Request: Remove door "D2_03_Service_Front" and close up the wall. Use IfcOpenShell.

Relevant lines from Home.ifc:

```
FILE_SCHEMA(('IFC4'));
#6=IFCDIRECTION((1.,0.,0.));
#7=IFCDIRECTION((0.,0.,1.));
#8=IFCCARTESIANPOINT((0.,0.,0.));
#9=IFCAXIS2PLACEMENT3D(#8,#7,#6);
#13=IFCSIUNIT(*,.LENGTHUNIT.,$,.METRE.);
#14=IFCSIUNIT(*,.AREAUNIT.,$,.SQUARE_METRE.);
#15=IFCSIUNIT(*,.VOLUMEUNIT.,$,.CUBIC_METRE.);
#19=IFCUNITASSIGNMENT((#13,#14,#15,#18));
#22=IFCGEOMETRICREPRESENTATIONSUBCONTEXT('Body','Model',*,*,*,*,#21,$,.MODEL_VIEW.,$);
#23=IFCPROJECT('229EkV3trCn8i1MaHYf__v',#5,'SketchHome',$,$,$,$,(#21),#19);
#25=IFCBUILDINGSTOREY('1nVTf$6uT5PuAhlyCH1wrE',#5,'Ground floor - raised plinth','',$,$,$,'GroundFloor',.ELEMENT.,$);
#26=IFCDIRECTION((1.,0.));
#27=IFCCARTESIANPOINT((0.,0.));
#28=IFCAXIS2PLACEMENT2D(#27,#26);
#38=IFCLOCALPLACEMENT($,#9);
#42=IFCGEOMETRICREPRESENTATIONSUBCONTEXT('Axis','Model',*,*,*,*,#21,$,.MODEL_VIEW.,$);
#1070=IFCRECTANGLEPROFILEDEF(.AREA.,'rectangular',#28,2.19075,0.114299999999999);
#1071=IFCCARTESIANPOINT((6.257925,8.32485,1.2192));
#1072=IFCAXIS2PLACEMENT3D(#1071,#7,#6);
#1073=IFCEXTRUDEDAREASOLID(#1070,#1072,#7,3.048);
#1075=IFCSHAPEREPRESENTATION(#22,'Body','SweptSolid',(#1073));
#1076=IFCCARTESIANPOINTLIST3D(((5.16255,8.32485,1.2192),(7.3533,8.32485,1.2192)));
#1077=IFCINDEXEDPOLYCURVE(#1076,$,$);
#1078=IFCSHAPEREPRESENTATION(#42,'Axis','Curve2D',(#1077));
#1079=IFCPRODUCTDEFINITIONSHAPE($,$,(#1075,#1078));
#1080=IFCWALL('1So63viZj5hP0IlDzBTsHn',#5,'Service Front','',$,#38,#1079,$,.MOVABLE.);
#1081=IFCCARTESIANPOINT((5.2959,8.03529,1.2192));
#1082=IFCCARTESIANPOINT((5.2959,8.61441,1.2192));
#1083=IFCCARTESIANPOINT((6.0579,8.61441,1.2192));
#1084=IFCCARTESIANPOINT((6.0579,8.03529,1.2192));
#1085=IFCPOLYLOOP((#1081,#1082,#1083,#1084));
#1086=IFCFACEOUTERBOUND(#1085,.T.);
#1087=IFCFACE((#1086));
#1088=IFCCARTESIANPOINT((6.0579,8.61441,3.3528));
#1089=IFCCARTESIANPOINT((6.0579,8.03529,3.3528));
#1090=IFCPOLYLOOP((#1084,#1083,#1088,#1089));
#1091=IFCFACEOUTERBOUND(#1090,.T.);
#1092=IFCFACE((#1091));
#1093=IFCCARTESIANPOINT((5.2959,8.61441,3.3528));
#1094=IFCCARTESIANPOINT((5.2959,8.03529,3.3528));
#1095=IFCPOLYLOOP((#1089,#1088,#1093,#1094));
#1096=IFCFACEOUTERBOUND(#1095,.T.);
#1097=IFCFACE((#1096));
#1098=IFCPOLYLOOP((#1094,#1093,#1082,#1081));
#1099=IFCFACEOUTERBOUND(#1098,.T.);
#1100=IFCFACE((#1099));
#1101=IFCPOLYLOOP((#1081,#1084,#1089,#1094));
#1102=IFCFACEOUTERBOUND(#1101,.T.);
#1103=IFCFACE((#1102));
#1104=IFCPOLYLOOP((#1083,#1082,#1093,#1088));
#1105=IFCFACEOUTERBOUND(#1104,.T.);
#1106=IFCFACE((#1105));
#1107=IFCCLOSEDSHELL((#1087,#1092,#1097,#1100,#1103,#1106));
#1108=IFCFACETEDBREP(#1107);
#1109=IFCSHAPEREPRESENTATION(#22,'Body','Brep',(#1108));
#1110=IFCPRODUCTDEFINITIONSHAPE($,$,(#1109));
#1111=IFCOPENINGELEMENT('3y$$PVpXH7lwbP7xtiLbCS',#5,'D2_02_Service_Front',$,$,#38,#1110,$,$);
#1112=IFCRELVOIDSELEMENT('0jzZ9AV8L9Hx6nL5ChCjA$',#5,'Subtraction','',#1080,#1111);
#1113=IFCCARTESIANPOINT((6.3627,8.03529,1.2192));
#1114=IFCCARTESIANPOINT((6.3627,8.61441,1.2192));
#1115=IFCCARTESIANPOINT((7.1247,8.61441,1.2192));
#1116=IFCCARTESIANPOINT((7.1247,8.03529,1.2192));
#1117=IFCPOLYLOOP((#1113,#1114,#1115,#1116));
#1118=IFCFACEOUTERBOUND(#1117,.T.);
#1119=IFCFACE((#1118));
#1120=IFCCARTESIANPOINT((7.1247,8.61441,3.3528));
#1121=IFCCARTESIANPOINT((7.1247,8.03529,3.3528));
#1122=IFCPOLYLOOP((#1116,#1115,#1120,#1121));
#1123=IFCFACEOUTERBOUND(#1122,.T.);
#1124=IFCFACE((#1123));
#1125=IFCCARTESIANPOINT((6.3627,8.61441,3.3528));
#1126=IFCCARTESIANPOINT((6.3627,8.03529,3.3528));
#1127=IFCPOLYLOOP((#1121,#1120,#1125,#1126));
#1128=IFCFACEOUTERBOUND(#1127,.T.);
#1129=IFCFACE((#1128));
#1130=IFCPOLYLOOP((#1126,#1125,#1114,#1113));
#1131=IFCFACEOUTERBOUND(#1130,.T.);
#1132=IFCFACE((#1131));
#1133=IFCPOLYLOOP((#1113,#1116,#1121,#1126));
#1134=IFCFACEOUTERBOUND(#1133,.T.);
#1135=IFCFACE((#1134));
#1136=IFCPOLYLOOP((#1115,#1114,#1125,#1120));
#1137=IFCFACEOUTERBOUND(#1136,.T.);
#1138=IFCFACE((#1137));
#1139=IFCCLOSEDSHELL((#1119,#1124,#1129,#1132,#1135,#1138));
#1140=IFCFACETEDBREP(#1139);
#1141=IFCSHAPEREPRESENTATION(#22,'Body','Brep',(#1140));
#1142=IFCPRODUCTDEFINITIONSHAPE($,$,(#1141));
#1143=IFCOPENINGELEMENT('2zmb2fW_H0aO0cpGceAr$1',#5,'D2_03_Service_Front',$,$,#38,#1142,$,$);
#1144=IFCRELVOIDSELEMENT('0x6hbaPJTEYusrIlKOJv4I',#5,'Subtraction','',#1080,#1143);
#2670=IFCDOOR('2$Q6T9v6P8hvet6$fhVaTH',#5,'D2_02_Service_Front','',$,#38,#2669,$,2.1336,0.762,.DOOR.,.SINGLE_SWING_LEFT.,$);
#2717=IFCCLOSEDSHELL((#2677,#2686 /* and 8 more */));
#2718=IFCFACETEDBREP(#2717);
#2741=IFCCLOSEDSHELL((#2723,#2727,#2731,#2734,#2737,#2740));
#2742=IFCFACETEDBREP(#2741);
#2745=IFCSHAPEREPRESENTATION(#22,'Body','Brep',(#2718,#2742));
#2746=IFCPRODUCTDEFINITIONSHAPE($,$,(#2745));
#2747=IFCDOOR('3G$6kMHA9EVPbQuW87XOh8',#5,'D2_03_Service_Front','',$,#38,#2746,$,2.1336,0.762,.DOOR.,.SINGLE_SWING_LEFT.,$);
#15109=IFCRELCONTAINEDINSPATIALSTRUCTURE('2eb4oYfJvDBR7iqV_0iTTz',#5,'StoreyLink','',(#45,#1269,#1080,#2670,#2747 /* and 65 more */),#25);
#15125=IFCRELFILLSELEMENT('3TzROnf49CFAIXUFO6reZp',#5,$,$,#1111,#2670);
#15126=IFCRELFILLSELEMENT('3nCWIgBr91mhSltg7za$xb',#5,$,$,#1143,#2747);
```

```python
import ifcopenshell
import ifcopenshell.api.feature
import ifcopenshell.api.root
import ifcopenshell.geom
import ifcopenshell.util.shape

model = ifcopenshell.open("Home.ifc")
settings = ifcopenshell.geom.settings()


def volume(element):
    """Net volume in cubic metres, openings subtracted."""
    shape = ifcopenshell.geom.create_shape(settings, element)
    return ifcopenshell.util.shape.get_volume(shape.geometry)


door = model.by_id(2747)
opening = door.FillsVoids[0].RelatingOpeningElement
wall = opening.VoidsElements[0].RelatingBuildingElement
before = volume(wall)

ifcopenshell.api.root.remove_product(model, product=door)
ifcopenshell.api.feature.remove_feature(model, feature=opening)

after = volume(wall)

print(f"wall volume {before:.3f} -> {after:.3f} m3")

model.write("Home_updated.ifc")
```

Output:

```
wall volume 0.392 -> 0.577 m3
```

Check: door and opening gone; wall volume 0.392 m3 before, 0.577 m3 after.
